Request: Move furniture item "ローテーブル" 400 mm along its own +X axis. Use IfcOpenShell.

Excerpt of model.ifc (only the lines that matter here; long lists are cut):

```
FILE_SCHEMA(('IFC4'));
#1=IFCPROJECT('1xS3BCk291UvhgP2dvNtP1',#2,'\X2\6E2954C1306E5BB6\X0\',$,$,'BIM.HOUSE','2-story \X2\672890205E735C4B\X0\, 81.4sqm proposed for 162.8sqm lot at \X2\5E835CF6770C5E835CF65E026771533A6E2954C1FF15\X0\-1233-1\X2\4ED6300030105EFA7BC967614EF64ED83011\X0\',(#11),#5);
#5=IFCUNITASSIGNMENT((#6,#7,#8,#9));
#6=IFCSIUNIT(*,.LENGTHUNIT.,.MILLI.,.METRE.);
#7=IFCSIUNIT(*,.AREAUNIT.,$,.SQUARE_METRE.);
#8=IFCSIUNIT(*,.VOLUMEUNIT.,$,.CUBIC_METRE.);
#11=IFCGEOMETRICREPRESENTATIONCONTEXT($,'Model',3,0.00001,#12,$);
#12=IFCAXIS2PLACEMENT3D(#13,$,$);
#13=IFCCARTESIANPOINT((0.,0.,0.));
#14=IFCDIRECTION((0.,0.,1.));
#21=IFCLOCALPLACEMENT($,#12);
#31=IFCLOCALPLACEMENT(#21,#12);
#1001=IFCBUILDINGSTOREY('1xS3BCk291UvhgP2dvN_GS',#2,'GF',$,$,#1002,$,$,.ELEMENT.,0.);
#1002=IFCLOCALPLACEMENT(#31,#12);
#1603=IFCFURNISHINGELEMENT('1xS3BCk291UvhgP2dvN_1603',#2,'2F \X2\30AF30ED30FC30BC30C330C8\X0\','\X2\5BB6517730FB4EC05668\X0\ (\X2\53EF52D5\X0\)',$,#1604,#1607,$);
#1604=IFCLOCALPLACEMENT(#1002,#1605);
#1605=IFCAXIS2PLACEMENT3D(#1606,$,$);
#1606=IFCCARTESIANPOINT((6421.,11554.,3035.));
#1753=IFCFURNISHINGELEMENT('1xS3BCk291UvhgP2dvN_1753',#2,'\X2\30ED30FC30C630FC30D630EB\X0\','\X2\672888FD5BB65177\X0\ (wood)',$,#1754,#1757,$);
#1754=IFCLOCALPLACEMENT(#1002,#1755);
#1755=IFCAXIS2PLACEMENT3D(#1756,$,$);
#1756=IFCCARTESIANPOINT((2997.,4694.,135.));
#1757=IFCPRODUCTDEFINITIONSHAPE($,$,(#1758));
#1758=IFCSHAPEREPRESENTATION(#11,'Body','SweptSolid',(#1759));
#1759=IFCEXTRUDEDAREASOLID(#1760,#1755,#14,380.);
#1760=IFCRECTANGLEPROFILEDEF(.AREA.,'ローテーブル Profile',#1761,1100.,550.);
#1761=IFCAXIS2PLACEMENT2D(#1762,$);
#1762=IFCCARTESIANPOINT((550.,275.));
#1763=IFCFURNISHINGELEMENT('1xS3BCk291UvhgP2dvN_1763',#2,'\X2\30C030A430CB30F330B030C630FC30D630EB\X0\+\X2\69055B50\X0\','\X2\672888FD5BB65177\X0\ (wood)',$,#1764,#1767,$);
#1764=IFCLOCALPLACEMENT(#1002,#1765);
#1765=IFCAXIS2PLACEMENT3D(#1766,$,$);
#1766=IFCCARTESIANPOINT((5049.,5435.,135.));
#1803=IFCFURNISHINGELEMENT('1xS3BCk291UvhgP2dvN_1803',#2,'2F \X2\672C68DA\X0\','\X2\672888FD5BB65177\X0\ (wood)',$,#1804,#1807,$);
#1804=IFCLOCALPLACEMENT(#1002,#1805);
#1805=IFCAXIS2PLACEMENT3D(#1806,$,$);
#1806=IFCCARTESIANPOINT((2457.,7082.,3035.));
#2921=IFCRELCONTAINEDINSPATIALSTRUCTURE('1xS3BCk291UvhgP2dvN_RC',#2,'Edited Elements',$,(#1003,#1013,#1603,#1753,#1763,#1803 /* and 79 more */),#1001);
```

```python
import ifcopenshell
import ifcopenshell.api.geometry
import ifcopenshell.util.placement
import ifcopenshell.util.unit

model = ifcopenshell.open("model.ifc")
unit_scale = ifcopenshell.util.unit.calculate_unit_scale(model)

item = model.by_guid("1xS3BCk291UvhgP2dvN_1753")
matrix = ifcopenshell.util.placement.get_local_placement(item.ObjectPlacement)
matrix[:3, 3] += matrix[:3, 0] * 0.4 / unit_scale
ifcopenshell.api.geometry.edit_object_placement(model, product=item, matrix=matrix, is_si=False)

print(ifcopenshell.util.placement.get_local_placement(item.ObjectPlacement).round(3) + 0.0)

model.write("model_updated.ifc")
```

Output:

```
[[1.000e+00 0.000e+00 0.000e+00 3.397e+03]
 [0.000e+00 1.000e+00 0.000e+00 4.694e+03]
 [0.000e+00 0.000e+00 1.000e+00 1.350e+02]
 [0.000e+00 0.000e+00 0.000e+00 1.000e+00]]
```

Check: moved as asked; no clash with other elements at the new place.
